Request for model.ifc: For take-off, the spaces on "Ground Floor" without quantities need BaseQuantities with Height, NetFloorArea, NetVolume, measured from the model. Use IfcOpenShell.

First a look at what the model holds.

```python
import ifcopenshell
import ifcopenshell.util.element
import ifcopenshell.util.unit

model = ifcopenshell.open("model.ifc")
print(model.schema)
for unit_type in ("LENGTHUNIT", "AREAUNIT", "VOLUMEUNIT"):
    print(unit_type, ifcopenshell.util.unit.calculate_unit_scale(model, unit_type))
storey = next(s for s in model.by_type("IfcBuildingStorey") if s.Name == "Ground Floor")
spaces = [e for e in ifcopenshell.util.element.get_decomposition(storey) if e.is_a("IfcSpace")]
for e in sorted(spaces, key=lambda e: e.id()):
    print(e.id(), e.is_a(), e.Name, list(ifcopenshell.util.element.get_psets(e, qtos_only=True)), sep=" | ")
```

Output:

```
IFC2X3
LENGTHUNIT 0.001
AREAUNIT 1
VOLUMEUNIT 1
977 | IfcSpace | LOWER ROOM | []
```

```python
import ifcopenshell
import ifcopenshell.api.pset
import ifcopenshell.geom
import ifcopenshell.util.element
import ifcopenshell.util.shape
import ifcopenshell.util.unit

model = ifcopenshell.open("model.ifc")
unit_scale = ifcopenshell.util.unit.calculate_unit_scale(model)
area_scale = ifcopenshell.util.unit.calculate_unit_scale(model, "AREAUNIT")
volume_scale = ifcopenshell.util.unit.calculate_unit_scale(model, "VOLUMEUNIT")
settings = ifcopenshell.geom.settings()

storey = next(s for s in model.by_type("IfcBuildingStorey") if s.Name == "Ground Floor")
spaces = [e for e in ifcopenshell.util.element.get_decomposition(storey) if e.is_a("IfcSpace")]

for e in sorted(spaces, key=lambda e: e.id()):
    if ifcopenshell.util.element.get_psets(e, qtos_only=True, should_inherit=False):
        continue
    # Geometry comes back in metres, in the element's own axes.
    shape = ifcopenshell.geom.create_shape(settings, e)
    values = {
        "Height": ifcopenshell.util.shape.get_z(shape.geometry) / unit_scale,
        "NetFloorArea": ifcopenshell.util.shape.get_footprint_area(shape.geometry) / area_scale,
        "NetVolume": ifcopenshell.util.shape.get_volume(shape.geometry) / volume_scale,
    }
    qto = ifcopenshell.api.pset.add_qto(model, product=e, name="BaseQuantities")
    ifcopenshell.api.pset.edit_qto(model, qto=qto, properties=values)
    print(e.id(), {k: round(v, 3) for k, v in values.items()})

model.write("model_rev.ifc")
```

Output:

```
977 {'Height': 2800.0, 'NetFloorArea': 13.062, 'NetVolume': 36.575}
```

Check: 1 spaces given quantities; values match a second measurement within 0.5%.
